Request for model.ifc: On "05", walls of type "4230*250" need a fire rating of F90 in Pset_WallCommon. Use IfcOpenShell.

First a look at what the model holds.

```python
import ifcopenshell
import ifcopenshell.util.element

model = ifcopenshell.open("model.ifc")
print(model.schema)
storey = next(s for s in model.by_type("IfcBuildingStorey") if s.Name == "05")
walls = [e for e in ifcopenshell.util.element.get_decomposition(storey) if e.is_a("IfcWall")]
seen = {}
for e in walls:
    element_type = ifcopenshell.util.element.get_type(e)
    key = (element_type.Name if element_type != e and element_type else None, ifcopenshell.util.element.get_pset(e, "Pset_WallCommon", "FireRating"))
    seen[key] = seen.get(key, 0) + 1
for (name, value), count in sorted(seen.items(), key=str):
    print(count, "x", name, "|", value)
```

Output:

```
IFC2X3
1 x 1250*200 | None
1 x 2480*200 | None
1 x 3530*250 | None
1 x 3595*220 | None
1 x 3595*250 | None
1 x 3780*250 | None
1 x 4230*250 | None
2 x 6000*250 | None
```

```python
import ifcopenshell
import ifcopenshell.api.pset
import ifcopenshell.util.element

model = ifcopenshell.open("model.ifc")

storey = next(s for s in model.by_type("IfcBuildingStorey") if s.Name == "05")
walls = [e for e in ifcopenshell.util.element.get_decomposition(storey) if e.is_a("IfcWall")]

count = 0
for e in walls:
    element_type = ifcopenshell.util.element.get_type(e)
    if element_type in (None, e) or element_type.Name != "4230*250":
        continue
    # add_pset returns the element's existing set when there is one.
    pset = ifcopenshell.api.pset.add_pset(model, product=e, name="Pset_WallCommon")
    ifcopenshell.api.pset.edit_pset(model, pset=pset, properties={"FireRating": "F90"})
    count += 1

print(count, "walls updated")

model.write("model_rev.ifc")
```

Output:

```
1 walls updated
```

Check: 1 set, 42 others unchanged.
